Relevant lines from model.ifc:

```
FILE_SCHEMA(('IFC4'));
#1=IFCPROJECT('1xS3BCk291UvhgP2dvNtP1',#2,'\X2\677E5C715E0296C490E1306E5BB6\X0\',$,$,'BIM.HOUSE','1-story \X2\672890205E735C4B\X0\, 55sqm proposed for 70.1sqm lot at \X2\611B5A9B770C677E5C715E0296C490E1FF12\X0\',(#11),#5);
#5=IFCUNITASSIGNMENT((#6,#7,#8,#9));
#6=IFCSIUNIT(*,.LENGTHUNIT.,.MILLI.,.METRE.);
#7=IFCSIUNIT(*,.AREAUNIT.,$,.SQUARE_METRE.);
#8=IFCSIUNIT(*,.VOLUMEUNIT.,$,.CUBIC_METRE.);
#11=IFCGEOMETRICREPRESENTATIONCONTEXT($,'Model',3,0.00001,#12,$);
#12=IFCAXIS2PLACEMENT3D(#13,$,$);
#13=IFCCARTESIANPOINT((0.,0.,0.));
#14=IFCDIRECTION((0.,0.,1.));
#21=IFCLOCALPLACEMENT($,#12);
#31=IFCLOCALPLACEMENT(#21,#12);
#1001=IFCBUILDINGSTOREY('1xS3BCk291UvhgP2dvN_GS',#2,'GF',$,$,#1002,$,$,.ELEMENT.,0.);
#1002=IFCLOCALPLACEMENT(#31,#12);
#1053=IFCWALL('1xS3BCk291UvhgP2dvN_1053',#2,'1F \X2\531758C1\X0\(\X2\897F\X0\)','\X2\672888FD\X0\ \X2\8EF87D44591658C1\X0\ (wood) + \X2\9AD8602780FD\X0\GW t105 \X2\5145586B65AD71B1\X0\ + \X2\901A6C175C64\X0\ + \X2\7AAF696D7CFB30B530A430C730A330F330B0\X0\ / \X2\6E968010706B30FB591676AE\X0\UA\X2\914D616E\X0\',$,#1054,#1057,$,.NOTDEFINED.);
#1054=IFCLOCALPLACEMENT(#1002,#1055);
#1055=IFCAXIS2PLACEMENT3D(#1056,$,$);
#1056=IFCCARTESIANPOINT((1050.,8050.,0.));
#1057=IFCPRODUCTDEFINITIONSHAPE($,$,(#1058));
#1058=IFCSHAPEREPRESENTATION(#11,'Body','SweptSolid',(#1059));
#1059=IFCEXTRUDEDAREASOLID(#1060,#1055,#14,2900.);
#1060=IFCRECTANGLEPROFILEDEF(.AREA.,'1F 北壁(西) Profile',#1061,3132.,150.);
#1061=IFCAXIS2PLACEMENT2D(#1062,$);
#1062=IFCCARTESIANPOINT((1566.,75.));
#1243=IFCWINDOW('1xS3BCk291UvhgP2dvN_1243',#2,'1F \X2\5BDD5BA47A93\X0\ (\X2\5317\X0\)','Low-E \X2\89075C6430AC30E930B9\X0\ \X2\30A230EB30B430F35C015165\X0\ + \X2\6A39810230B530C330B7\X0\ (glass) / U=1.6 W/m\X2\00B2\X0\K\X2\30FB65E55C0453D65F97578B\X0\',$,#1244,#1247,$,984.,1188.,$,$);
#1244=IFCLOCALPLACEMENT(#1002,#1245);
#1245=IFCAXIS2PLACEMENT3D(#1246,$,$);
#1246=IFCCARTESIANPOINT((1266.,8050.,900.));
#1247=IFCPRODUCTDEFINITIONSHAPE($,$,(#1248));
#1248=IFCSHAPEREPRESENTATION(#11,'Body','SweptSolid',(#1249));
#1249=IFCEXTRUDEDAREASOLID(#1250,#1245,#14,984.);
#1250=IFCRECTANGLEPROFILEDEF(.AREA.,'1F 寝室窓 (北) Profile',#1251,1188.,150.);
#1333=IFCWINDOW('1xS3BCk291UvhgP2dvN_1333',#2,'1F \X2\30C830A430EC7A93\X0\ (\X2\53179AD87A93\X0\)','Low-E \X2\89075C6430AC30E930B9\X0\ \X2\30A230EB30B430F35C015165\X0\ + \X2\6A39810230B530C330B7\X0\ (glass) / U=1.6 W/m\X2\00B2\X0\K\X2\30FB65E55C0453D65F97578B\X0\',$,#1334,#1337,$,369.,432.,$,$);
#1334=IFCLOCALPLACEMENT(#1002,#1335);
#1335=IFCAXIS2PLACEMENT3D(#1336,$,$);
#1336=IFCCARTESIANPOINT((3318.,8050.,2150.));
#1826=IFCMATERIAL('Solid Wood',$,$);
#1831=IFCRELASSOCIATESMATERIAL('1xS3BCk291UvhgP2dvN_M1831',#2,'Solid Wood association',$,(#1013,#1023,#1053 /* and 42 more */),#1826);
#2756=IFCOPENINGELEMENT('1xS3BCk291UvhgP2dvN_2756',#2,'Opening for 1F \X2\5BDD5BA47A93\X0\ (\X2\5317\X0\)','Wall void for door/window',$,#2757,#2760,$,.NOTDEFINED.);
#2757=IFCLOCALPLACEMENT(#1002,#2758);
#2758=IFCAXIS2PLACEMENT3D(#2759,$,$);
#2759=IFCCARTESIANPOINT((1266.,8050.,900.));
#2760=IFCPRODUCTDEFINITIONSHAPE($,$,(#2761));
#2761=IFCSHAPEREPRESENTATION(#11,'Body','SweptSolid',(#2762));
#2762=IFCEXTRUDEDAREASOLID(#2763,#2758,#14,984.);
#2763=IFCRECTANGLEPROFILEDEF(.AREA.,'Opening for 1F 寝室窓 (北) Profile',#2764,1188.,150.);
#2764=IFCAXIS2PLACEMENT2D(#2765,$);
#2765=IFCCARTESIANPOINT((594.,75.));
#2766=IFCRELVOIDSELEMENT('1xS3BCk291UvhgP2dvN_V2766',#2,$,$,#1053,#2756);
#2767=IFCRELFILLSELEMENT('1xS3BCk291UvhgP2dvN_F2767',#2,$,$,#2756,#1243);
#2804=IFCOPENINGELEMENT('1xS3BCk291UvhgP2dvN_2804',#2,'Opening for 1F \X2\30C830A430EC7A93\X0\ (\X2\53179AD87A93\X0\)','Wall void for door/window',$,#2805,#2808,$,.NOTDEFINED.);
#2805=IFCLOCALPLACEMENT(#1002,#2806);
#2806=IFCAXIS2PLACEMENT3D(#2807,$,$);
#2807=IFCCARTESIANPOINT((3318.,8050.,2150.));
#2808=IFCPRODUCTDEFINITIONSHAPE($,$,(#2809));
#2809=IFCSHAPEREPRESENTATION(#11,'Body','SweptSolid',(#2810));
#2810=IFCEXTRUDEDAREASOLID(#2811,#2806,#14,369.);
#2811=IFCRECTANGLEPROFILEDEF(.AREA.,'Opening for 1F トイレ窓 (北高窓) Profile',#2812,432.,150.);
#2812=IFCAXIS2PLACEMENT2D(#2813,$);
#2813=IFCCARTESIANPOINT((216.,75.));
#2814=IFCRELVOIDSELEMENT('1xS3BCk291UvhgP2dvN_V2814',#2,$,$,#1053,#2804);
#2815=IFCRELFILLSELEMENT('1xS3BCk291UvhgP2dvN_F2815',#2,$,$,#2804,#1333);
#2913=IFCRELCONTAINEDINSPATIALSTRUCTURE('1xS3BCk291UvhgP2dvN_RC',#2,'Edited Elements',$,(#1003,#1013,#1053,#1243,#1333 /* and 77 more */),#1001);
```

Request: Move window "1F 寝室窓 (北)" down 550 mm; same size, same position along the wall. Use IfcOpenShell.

```python
import numpy as np
import ifcopenshell
import ifcopenshell.api.geometry
import ifcopenshell.util.placement
import ifcopenshell.util.unit

model = ifcopenshell.open("model.ifc")
unit_scale = ifcopenshell.util.unit.calculate_unit_scale(model)

window = model.by_id(1243)
opening = window.FillsVoids[0].RelatingOpeningElement
dz = -0.55 / unit_scale

shift = np.array([0.0, 0.0, dz])
# The window is not placed relative to its opening, so move both.
for product in (opening, window):
    matrix = ifcopenshell.util.placement.get_local_placement(product.ObjectPlacement)
    matrix[:3, 3] += shift
    ifcopenshell.api.geometry.edit_object_placement(model, product=product, matrix=matrix, is_si=False)

print(f"moved by {dz * unit_scale:+.3f} m")

model.write("model_updated.ifc")
```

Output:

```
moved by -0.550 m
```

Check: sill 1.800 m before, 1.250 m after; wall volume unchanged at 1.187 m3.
